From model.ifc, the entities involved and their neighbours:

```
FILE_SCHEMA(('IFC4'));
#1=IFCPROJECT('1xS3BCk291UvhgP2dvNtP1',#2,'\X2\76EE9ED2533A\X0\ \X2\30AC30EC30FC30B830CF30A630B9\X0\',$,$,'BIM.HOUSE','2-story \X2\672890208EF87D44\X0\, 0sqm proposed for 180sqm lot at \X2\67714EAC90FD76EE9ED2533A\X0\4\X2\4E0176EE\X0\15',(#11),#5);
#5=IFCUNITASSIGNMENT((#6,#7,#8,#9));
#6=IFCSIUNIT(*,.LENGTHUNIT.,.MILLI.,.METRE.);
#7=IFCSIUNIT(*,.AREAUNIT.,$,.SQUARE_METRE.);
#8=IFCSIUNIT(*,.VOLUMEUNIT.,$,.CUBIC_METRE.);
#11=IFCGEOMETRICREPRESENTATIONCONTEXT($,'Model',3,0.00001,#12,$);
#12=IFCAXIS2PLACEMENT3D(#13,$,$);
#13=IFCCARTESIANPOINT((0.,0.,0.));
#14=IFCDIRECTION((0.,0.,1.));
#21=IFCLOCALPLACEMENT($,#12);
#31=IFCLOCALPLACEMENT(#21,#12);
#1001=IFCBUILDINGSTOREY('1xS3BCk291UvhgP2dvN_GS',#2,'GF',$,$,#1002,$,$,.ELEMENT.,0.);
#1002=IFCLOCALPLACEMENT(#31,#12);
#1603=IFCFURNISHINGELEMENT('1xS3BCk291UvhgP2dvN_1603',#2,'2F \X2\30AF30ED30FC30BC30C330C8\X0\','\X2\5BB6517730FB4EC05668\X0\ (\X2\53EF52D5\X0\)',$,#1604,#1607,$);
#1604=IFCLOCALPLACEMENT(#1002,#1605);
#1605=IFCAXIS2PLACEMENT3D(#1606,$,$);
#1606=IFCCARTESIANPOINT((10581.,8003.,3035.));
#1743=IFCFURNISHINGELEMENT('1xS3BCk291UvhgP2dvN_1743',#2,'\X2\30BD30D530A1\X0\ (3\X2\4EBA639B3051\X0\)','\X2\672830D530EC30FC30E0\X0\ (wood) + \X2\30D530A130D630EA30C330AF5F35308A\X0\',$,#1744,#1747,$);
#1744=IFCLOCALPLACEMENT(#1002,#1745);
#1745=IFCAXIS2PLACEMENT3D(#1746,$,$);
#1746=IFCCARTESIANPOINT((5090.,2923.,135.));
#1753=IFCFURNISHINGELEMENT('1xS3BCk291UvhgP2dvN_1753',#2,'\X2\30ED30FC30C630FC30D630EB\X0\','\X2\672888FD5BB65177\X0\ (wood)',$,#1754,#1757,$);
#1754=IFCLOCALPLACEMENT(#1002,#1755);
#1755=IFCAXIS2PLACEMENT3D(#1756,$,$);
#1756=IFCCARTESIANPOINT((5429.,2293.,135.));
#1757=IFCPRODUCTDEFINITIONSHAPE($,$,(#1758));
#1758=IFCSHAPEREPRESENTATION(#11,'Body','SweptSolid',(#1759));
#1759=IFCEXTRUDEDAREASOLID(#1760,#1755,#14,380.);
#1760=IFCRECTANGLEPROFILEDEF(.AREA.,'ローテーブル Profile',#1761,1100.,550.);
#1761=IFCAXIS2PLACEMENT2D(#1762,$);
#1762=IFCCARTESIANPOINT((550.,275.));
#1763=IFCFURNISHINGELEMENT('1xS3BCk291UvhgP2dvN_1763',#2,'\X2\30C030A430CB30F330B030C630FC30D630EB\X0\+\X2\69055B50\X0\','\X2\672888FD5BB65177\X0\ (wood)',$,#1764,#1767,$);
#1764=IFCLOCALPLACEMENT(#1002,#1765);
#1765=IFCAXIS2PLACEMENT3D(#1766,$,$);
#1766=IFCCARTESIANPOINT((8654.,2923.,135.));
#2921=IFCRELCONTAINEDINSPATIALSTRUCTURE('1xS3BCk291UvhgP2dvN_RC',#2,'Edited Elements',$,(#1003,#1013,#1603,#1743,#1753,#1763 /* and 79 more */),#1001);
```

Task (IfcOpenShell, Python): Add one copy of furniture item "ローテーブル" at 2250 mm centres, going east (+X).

```python
import numpy as np
import ifcopenshell
import ifcopenshell.api.geometry
import ifcopenshell.api.root
import ifcopenshell.util.element
import ifcopenshell.util.placement
import ifcopenshell.util.unit

model = ifcopenshell.open("model.ifc")
unit_scale = ifcopenshell.util.unit.calculate_unit_scale(model)


def reuse_history(source, copy):
    """copy_class also copies each property set's owner history, people and application; keep the originals."""
    for rel in copy.IsDefinedBy:
        if rel.is_a("IfcRelDefinesByProperties") and (history := rel.RelatingPropertyDefinition.OwnerHistory):
            rel.RelatingPropertyDefinition.OwnerHistory = source.OwnerHistory
            ifcopenshell.util.element.remove_deep2(model, history)


source = model.by_id(1753)
base = ifcopenshell.util.placement.get_local_placement(source.ObjectPlacement)
step = np.array([1.0, 0.0, 0.0]) * 2.25 / unit_scale

for i in range(1, 2):
    copy = ifcopenshell.api.root.copy_class(model, product=source)
    copy.Representation = ifcopenshell.util.element.copy_deep(
        model, source.Representation, exclude=["IfcGeometricRepresentationContext", "IfcRepresentationMap"]
    )
    reuse_history(source, copy)
    matrix = base.copy()
    matrix[:3, 3] += i * step
    print("added at", matrix[:3, 3].round(3) + 0.0)
    ifcopenshell.api.geometry.edit_object_placement(model, product=copy, matrix=matrix, is_si=False)

model.write("model_edited.ifc")
```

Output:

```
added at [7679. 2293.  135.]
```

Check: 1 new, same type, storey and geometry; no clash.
